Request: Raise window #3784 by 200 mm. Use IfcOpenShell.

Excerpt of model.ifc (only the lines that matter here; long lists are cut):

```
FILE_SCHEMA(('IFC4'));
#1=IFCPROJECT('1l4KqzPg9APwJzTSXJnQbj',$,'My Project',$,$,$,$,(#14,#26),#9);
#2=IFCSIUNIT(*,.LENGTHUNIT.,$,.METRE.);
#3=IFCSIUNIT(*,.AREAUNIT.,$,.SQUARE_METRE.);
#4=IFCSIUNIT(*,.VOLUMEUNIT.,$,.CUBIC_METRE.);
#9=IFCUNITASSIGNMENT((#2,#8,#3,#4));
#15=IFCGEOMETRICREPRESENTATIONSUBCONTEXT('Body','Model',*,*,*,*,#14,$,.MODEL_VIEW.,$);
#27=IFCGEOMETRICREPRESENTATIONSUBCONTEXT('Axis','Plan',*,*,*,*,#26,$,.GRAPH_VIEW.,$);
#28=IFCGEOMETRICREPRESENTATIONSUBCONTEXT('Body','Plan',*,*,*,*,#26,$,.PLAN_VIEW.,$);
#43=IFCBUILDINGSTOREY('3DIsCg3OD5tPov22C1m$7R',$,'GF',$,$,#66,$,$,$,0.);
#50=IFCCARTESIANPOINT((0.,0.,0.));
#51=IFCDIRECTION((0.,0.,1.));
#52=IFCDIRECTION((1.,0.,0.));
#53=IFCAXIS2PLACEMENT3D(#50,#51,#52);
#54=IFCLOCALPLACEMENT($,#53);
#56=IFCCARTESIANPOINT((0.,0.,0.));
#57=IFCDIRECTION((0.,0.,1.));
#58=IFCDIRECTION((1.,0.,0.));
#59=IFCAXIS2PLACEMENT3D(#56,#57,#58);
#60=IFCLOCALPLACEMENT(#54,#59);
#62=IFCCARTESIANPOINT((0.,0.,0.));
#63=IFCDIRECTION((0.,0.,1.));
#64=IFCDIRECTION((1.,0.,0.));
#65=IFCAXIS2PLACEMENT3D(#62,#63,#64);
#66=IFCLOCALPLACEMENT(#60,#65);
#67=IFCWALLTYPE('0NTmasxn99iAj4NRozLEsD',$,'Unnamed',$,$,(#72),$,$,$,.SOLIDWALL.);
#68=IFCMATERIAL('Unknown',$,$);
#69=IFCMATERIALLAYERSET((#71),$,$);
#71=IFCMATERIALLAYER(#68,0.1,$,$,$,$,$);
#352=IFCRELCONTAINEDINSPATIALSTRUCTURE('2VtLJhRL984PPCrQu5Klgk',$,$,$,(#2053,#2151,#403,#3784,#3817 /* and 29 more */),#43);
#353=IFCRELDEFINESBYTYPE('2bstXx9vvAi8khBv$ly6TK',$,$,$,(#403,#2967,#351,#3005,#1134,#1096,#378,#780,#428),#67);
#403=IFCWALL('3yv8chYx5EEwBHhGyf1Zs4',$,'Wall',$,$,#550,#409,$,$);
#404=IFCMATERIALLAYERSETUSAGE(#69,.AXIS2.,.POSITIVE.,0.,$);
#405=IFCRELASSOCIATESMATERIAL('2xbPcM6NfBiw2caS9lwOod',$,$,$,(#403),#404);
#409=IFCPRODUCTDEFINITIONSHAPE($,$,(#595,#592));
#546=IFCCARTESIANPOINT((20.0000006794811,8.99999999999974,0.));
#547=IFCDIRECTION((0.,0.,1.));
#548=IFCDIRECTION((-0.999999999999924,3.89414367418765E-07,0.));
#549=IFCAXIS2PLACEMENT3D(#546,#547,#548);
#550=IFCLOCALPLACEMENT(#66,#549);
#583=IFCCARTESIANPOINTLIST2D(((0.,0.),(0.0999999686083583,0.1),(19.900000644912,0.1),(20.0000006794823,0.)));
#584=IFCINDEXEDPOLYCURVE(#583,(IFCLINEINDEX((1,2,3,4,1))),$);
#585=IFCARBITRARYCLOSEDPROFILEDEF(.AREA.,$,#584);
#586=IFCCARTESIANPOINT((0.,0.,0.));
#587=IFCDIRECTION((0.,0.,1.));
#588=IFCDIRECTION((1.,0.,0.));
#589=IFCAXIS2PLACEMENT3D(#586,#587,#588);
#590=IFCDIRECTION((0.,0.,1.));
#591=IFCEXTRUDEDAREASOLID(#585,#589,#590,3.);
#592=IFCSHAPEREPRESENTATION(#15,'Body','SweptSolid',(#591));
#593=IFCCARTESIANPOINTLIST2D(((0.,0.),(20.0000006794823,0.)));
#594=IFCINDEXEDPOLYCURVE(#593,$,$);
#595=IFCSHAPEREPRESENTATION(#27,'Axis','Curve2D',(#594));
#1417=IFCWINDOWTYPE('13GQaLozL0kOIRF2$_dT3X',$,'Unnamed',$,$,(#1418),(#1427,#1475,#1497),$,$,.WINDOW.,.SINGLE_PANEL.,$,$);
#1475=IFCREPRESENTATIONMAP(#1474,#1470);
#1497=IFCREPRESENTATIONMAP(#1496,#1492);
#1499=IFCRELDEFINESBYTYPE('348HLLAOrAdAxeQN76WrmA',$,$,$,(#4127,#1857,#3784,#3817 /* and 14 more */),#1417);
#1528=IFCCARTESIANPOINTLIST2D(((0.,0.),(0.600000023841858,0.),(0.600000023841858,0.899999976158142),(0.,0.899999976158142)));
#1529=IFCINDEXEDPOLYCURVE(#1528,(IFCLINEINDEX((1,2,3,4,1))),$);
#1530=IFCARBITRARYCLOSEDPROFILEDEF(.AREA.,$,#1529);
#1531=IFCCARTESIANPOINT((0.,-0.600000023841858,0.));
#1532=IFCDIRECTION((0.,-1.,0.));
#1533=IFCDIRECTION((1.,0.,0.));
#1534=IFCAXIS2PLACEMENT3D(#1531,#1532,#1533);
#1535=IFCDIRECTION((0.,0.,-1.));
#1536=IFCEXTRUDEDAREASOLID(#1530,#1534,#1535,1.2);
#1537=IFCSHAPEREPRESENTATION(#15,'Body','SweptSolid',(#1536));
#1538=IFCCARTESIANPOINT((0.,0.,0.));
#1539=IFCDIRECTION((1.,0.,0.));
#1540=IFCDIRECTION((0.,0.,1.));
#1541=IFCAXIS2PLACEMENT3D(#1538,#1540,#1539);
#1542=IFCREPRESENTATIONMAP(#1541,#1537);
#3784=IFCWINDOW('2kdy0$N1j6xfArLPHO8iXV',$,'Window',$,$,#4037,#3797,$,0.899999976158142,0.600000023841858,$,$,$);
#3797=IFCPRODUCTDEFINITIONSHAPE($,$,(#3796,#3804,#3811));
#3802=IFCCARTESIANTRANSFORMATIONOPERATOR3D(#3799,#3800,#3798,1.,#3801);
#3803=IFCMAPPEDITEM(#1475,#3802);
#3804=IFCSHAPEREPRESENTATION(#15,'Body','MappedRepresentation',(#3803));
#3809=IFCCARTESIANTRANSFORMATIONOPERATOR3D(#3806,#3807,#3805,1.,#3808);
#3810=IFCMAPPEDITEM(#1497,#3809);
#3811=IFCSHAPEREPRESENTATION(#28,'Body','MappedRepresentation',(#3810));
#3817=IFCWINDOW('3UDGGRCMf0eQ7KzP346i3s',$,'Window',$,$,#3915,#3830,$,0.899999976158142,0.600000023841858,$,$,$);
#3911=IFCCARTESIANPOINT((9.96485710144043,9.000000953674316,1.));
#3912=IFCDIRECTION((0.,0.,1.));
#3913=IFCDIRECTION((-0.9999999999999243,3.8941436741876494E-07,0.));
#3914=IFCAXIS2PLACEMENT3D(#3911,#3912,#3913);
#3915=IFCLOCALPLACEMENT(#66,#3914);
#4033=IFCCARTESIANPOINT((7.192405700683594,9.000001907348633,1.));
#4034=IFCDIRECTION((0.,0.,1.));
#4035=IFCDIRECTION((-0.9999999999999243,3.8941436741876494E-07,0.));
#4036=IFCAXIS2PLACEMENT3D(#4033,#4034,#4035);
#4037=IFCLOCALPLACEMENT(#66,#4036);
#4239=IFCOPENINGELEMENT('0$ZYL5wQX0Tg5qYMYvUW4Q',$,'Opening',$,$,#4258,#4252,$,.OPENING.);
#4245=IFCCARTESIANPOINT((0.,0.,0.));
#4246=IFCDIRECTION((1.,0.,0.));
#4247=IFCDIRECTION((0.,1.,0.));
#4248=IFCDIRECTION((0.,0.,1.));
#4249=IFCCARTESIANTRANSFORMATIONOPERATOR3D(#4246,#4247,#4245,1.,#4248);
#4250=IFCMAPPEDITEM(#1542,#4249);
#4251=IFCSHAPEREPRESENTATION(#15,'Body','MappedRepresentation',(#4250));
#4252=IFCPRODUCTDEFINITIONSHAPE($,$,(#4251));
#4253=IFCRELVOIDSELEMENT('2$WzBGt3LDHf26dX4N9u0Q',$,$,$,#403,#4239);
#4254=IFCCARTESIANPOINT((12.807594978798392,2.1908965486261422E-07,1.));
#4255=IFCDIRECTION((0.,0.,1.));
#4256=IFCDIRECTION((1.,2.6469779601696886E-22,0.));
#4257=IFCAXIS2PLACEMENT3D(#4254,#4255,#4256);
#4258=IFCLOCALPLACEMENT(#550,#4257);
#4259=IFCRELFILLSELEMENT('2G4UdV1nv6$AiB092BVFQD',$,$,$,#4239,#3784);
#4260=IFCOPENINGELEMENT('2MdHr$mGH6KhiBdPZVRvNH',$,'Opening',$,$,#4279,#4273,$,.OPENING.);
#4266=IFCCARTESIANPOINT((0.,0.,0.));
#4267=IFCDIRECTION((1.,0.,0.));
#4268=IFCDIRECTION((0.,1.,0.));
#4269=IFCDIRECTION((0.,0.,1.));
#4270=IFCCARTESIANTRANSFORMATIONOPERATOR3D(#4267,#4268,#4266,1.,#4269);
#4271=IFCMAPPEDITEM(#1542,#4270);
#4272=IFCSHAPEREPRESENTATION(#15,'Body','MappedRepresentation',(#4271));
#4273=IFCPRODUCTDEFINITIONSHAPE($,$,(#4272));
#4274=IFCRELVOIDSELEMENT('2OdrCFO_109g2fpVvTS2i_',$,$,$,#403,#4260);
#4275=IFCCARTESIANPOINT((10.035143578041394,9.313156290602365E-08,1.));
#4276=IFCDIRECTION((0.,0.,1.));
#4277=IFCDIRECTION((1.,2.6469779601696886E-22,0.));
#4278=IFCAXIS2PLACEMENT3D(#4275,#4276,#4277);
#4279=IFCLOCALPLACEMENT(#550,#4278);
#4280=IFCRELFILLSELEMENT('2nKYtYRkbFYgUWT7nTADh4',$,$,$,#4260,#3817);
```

```python
import numpy as np
import ifcopenshell
import ifcopenshell.api.geometry
import ifcopenshell.util.placement
import ifcopenshell.util.unit

model = ifcopenshell.open("model.ifc")
unit_scale = ifcopenshell.util.unit.calculate_unit_scale(model)

window = model.by_guid("2kdy0$N1j6xfArLPHO8iXV")
opening = window.FillsVoids[0].RelatingOpeningElement
dz = 0.2

shift = np.array([0.0, 0.0, dz])
# The window is not placed relative to its opening, so move both.
for product in (opening, window):
    matrix = ifcopenshell.util.placement.get_local_placement(product.ObjectPlacement)
    matrix[:3, 3] += shift
    ifcopenshell.api.geometry.edit_object_placement(model, product=product, matrix=matrix, is_si=False)

print(f"moved by {dz * unit_scale:+.3f} m")

model.write("model_v2.ifc")
```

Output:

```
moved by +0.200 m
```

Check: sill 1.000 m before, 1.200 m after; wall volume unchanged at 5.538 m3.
